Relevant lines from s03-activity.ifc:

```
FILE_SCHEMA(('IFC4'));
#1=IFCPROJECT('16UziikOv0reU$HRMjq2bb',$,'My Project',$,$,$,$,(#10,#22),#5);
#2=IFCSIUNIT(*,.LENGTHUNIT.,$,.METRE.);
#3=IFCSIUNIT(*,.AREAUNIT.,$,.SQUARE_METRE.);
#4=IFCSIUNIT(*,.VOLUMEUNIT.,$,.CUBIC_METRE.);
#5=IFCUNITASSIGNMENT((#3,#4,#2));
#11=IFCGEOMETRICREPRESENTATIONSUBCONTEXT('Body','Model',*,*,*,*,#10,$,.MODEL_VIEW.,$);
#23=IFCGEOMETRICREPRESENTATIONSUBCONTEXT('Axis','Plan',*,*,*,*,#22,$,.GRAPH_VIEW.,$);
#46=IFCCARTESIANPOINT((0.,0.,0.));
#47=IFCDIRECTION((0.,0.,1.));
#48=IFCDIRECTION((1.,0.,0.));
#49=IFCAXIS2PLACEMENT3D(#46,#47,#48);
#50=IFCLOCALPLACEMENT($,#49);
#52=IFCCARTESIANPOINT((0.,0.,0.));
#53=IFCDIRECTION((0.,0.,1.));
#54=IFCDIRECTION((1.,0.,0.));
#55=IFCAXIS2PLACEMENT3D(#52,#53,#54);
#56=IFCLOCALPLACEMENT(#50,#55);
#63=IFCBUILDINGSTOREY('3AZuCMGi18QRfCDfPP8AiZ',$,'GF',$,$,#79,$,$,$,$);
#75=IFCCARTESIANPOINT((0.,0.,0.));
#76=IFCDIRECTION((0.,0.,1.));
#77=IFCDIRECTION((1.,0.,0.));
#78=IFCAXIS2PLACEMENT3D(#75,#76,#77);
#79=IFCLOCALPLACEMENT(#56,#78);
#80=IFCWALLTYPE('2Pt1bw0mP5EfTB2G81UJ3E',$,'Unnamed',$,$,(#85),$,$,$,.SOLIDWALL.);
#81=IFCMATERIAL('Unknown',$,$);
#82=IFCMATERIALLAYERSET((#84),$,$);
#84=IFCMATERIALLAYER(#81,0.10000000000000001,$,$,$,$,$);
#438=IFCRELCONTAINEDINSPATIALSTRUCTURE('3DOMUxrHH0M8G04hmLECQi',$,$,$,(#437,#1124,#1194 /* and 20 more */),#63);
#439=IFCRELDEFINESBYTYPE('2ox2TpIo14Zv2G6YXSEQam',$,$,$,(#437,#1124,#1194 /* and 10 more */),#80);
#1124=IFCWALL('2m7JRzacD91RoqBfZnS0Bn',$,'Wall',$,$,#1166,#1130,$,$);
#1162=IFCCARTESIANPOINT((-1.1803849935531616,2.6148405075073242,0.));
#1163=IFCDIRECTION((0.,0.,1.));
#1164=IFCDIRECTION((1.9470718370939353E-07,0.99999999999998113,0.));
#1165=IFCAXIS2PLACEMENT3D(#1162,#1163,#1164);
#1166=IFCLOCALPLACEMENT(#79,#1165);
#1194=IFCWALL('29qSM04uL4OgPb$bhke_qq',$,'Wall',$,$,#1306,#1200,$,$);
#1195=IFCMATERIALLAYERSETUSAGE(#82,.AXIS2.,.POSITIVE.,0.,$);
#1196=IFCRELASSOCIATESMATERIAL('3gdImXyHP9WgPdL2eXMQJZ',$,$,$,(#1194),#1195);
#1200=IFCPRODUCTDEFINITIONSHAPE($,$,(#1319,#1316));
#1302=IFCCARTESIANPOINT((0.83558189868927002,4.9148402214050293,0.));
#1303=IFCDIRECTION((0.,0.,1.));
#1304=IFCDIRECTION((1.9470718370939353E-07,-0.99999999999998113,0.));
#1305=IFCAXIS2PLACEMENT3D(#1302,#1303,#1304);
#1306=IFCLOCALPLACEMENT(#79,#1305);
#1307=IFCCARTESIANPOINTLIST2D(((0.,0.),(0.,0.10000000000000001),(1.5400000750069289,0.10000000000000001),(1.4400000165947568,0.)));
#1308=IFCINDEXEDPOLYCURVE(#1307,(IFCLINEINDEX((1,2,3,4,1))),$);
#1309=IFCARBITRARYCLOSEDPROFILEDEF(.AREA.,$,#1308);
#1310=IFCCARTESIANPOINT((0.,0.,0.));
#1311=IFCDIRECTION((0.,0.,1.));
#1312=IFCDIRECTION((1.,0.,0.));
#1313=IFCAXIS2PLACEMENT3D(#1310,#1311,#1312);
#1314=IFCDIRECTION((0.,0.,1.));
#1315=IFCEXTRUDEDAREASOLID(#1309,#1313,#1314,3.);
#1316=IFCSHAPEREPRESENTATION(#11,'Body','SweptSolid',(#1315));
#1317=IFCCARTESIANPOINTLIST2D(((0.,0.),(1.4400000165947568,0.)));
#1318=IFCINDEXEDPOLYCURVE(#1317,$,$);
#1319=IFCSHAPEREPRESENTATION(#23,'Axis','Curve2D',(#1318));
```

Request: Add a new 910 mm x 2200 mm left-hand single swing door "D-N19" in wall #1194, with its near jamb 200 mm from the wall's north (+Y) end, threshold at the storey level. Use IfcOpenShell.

```python
import numpy as np
import ifcopenshell
import ifcopenshell.api.feature
import ifcopenshell.api.geometry
import ifcopenshell.api.root
import ifcopenshell.api.spatial
import ifcopenshell.geom
import ifcopenshell.util.element
import ifcopenshell.util.placement
import ifcopenshell.util.representation
import ifcopenshell.util.shape
import ifcopenshell.util.unit

model = ifcopenshell.open("s03-activity.ifc")
unit_scale = ifcopenshell.util.unit.calculate_unit_scale(model)
settings = ifcopenshell.geom.settings()


def volume(element):
    """Net volume in cubic metres, openings subtracted."""
    shape = ifcopenshell.geom.create_shape(settings, element)
    return ifcopenshell.util.shape.get_volume(shape.geometry)


wall = model.by_id(1194)
storey = ifcopenshell.util.element.get_container(wall, ifc_class="IfcBuildingStorey")
context = ifcopenshell.util.representation.get_context(model, "Model", "Body", "MODEL_VIEW")
before = volume(wall)

width, height, from_end, sill = 0.91, 2.2, 0.2, 0.0  # metres

# The wall runs along its own X axis, and the end named is its -X end.
wall_shape = ifcopenshell.geom.create_shape(settings, wall)
x, y, z = ifcopenshell.util.shape.get_vertices(wall_shape.geometry).T
start = x.min() + from_end
face, thickness = float(y.min()), float(y.max() - y.min())
wall_matrix = ifcopenshell.util.placement.get_local_placement(wall.ObjectPlacement)
level = ifcopenshell.util.placement.get_local_placement(storey.ObjectPlacement)[2, 3]


def in_wall(x, y):
    """Placement at x, y metres in the wall's axes, at sill height."""
    matrix = wall_matrix.copy()
    matrix[:, 3] = wall_matrix @ np.array([x / unit_scale, y / unit_scale, 0.0, 1.0])
    matrix[2, 3] = level + sill / unit_scale
    return matrix


# Opening: a box that overshoots both wall faces by 50 mm.
opening = ifcopenshell.api.root.create_entity(model, ifc_class="IfcOpeningElement", predefined_type="OPENING")
box = ifcopenshell.api.geometry.add_wall_representation(
    model, context=context, length=width, height=height, thickness=thickness + 0.1
)
ifcopenshell.api.geometry.assign_representation(model, product=opening, representation=box)
ifcopenshell.api.geometry.edit_object_placement(model, product=opening, matrix=in_wall(start, face - 0.05), is_si=False)
ifcopenshell.api.feature.add_feature(model, feature=opening, element=wall)

door = ifcopenshell.api.root.create_entity(model, ifc_class="IfcDoor", name="D-N19", predefined_type="DOOR")
door.OverallWidth, door.OverallHeight = width / unit_scale, height / unit_scale
door.OperationType = "SINGLE_SWING_LEFT"
body = ifcopenshell.api.geometry.add_door_representation(
    model,
    context=context,
    overall_width=door.OverallWidth,
    overall_height=door.OverallHeight,
    operation_type="SINGLE_SWING_LEFT",
    lining_properties={"LiningDepth": thickness / unit_scale, "ThresholdDepth": thickness / unit_scale},
)
ifcopenshell.api.geometry.assign_representation(model, product=door, representation=body)
ifcopenshell.api.spatial.assign_container(model, products=[door], relating_structure=storey)
ifcopenshell.api.feature.add_filling(model, opening=opening, element=door)

# The lining spans the wall, so the door starts at the wall face.
ifcopenshell.api.geometry.edit_object_placement(model, product=door, matrix=in_wall(start, face), is_si=False)

after = volume(wall)

print(f"wall volume {before:.3f} -> {after:.3f} m3")

model.write("s03-activity-out.ifc")
```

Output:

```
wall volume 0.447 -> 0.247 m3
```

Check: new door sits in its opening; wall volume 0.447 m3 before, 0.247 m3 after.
